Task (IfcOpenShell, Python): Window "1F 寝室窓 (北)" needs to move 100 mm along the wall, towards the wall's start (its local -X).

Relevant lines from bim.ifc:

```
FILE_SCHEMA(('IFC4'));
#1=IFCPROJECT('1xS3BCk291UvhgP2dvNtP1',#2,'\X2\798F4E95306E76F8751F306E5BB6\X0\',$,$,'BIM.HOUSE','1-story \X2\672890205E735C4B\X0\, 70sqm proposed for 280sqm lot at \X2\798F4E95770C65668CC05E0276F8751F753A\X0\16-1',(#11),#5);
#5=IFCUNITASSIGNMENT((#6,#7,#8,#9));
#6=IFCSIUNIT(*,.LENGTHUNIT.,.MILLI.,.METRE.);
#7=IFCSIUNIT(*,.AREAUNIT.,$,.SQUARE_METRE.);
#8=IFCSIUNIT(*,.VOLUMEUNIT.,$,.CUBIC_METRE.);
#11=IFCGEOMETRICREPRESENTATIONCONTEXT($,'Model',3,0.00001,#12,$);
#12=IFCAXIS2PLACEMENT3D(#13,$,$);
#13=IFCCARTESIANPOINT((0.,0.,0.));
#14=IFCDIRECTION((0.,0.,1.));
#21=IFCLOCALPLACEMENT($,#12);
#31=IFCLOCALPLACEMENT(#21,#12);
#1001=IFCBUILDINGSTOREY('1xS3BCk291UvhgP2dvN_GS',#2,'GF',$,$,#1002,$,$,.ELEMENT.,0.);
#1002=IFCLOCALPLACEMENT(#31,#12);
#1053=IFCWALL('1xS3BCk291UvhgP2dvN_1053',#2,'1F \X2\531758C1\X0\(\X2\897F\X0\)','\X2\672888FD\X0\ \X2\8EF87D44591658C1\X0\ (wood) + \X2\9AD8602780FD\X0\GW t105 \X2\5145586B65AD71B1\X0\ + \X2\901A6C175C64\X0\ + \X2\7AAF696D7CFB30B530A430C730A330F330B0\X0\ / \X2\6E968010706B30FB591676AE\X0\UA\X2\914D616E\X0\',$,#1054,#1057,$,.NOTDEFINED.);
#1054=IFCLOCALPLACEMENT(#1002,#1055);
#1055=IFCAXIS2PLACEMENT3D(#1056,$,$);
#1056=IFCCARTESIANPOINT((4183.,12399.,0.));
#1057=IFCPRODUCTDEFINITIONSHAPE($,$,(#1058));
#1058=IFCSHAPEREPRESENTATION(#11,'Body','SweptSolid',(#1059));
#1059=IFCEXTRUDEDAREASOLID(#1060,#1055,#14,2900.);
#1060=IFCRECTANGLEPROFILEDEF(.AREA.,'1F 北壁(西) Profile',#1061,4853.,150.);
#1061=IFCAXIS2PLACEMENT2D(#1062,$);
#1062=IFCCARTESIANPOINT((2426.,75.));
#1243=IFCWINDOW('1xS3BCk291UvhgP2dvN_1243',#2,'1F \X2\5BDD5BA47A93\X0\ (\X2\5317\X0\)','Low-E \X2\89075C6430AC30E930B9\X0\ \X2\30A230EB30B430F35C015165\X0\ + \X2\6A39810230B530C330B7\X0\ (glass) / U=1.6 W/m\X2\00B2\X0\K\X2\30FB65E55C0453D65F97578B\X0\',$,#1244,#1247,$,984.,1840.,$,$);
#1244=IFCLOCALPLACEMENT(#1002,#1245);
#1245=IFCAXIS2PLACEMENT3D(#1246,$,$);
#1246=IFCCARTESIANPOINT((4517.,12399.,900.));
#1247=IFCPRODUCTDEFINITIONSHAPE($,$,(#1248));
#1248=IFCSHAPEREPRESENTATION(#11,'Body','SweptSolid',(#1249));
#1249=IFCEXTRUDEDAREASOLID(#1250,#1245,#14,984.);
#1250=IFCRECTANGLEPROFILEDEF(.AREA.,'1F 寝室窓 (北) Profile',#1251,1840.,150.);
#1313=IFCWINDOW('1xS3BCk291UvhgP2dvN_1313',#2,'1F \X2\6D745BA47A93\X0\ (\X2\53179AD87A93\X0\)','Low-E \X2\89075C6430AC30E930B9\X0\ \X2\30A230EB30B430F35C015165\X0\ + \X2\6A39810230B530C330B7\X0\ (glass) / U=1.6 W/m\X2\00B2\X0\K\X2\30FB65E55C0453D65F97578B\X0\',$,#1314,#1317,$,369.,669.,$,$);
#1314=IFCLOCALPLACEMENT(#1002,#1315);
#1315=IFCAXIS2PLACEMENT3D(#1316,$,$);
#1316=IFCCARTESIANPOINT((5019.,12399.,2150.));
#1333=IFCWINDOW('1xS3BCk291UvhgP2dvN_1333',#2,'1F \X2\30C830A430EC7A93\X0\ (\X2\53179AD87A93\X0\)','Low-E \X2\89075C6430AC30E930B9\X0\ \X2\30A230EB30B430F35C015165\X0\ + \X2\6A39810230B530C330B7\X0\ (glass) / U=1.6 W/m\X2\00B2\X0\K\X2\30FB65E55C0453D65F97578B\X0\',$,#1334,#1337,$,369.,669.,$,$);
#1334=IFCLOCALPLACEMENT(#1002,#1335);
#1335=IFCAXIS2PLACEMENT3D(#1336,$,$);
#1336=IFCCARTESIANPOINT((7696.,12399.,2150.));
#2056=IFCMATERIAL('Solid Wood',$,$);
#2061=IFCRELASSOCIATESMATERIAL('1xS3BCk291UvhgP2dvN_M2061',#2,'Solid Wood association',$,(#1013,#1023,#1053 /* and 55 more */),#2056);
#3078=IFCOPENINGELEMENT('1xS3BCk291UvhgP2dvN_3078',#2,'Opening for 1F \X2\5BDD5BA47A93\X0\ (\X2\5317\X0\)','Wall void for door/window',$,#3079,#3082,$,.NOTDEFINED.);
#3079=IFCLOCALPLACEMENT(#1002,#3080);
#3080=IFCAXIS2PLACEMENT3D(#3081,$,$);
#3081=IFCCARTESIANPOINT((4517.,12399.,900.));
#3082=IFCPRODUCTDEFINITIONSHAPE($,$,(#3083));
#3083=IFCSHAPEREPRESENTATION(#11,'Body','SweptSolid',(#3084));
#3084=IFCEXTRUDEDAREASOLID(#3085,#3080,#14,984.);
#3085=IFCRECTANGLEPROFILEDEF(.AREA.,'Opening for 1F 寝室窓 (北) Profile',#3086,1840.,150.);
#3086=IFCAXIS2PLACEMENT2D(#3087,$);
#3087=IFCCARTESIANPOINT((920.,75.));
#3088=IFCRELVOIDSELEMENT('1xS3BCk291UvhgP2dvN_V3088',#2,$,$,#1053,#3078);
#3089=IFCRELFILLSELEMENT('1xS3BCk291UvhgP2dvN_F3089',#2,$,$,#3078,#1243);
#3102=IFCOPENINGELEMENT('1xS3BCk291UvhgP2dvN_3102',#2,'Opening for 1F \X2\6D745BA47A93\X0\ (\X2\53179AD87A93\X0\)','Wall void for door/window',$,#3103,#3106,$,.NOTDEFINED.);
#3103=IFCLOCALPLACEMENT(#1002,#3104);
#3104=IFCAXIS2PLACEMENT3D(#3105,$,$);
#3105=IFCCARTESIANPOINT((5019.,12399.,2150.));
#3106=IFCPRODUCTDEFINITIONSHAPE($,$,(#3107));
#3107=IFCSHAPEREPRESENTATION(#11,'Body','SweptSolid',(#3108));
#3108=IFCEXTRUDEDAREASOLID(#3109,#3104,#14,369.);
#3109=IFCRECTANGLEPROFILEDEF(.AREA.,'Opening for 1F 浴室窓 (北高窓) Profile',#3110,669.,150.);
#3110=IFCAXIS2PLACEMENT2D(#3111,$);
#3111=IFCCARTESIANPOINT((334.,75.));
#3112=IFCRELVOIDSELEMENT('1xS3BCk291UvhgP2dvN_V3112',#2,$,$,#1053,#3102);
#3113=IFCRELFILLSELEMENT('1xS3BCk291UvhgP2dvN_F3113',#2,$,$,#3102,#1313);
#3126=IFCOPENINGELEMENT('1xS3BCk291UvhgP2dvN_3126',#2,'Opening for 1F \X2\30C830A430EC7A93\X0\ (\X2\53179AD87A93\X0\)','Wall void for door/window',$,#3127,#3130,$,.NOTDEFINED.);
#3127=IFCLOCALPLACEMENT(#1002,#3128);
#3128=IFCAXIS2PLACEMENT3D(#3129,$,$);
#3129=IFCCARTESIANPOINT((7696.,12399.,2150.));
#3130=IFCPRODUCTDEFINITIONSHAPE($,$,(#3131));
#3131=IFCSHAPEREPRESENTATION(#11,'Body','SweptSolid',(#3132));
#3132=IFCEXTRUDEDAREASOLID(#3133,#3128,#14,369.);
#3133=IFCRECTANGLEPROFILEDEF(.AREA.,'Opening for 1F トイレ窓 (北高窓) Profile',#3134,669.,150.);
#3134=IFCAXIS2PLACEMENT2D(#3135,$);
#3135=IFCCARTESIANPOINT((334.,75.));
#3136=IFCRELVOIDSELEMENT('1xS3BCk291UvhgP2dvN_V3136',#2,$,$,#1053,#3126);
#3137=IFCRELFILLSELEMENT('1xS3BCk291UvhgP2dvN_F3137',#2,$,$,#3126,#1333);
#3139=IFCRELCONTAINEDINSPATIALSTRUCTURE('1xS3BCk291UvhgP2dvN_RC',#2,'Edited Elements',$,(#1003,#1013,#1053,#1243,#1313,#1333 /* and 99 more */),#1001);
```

```python
import ifcopenshell
import ifcopenshell.api.geometry
import ifcopenshell.util.placement
import ifcopenshell.util.unit

model = ifcopenshell.open("bim.ifc")
unit_scale = ifcopenshell.util.unit.calculate_unit_scale(model)

window = model.by_id(1243)
opening = window.FillsVoids[0].RelatingOpeningElement
wall = opening.VoidsElements[0].RelatingBuildingElement

wall_matrix = ifcopenshell.util.placement.get_local_placement(wall.ObjectPlacement)
shift = wall_matrix[:3, 0] * -0.1 / unit_scale
before = ifcopenshell.util.placement.get_local_placement(window.ObjectPlacement)[:3, 3].copy()

# The window is not placed relative to its opening, so move both.
for product in (opening, window):
    matrix = ifcopenshell.util.placement.get_local_placement(product.ObjectPlacement)
    matrix[:3, 3] += shift
    ifcopenshell.api.geometry.edit_object_placement(model, product=product, matrix=matrix, is_si=False)

after = ifcopenshell.util.placement.get_local_placement(window.ObjectPlacement)[:3, 3]
print("window moved by", (after - before).round(3) + 0.0)

model.write("bim_v2.ifc")
```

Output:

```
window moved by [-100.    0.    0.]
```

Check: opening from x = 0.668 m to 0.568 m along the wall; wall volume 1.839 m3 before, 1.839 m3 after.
